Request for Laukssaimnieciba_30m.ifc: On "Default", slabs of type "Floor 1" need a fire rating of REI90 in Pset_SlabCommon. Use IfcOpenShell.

First a look at what the model holds.

```python
import ifcopenshell
import ifcopenshell.util.element

model = ifcopenshell.open("Laukssaimnieciba_30m.ifc")
print(model.schema)
storey = next(s for s in model.by_type("IfcBuildingStorey") if s.Name == "Default")
slabs = [e for e in ifcopenshell.util.element.get_decomposition(storey) if e.is_a("IfcSlab")]
seen = {}
for e in slabs:
    element_type = ifcopenshell.util.element.get_type(e)
    key = (element_type.Name if element_type != e and element_type else None, ifcopenshell.util.element.get_pset(e, "Pset_SlabCommon", "FireRating"))
    seen[key] = seen.get(key, 0) + 1
for (name, value), count in sorted(seen.items(), key=str):
    print(count, "x", name, "|", value)
```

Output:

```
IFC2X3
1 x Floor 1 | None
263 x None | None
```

```python
import ifcopenshell
import ifcopenshell.api.pset
import ifcopenshell.util.element

model = ifcopenshell.open("Laukssaimnieciba_30m.ifc")

storey = next(s for s in model.by_type("IfcBuildingStorey") if s.Name == "Default")
slabs = [e for e in ifcopenshell.util.element.get_decomposition(storey) if e.is_a("IfcSlab")]

count = 0
for e in slabs:
    element_type = ifcopenshell.util.element.get_type(e)
    if element_type in (None, e) or element_type.Name != "Floor 1":
        continue
    # add_pset returns the element's existing set when there is one.
    pset = ifcopenshell.api.pset.add_pset(model, product=e, name="Pset_SlabCommon")
    ifcopenshell.api.pset.edit_pset(model, pset=pset, properties={"FireRating": "REI90"})
    count += 1

print(count, "slabs updated")

model.write("Laukssaimnieciba_30m_v2.ifc")
```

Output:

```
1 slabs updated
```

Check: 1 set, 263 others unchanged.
